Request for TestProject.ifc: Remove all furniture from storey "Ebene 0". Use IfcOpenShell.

First a look at what the model holds.

```python
import ifcopenshell
import ifcopenshell.util.element

model = ifcopenshell.open("TestProject.ifc")
print(model.schema)
storey = next(s for s in model.by_type("IfcBuildingStorey") if s.Name == "Ebene 0")
furniture = [e for e in ifcopenshell.util.element.get_decomposition(storey) if e.is_a("IfcFurnishingElement")]
seen = {}
for e in furniture:
    element_type = ifcopenshell.util.element.get_type(e)
    name = element_type.Name if element_type not in (None, e) else None
    seen[name] = seen.get(name, 0) + 1
for name, count in sorted(seen.items(), key=str):
    print(count, "x", name)
```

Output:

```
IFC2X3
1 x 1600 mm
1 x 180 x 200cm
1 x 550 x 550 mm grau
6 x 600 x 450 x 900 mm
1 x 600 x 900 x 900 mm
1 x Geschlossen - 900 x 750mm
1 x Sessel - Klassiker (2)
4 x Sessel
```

```python
import ifcopenshell
import ifcopenshell.api.root
import ifcopenshell.util.element

model = ifcopenshell.open("TestProject.ifc")

storey = next(s for s in model.by_type("IfcBuildingStorey") if s.Name == "Ebene 0")
furniture = [e for e in ifcopenshell.util.element.get_decomposition(storey) if e.is_a("IfcFurnishingElement")]

for e in furniture:
    ifcopenshell.api.root.remove_product(model, product=e)
print(len(furniture), "removed")

model.write("TestProject_edited.ifc")
```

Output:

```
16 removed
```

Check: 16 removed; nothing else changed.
